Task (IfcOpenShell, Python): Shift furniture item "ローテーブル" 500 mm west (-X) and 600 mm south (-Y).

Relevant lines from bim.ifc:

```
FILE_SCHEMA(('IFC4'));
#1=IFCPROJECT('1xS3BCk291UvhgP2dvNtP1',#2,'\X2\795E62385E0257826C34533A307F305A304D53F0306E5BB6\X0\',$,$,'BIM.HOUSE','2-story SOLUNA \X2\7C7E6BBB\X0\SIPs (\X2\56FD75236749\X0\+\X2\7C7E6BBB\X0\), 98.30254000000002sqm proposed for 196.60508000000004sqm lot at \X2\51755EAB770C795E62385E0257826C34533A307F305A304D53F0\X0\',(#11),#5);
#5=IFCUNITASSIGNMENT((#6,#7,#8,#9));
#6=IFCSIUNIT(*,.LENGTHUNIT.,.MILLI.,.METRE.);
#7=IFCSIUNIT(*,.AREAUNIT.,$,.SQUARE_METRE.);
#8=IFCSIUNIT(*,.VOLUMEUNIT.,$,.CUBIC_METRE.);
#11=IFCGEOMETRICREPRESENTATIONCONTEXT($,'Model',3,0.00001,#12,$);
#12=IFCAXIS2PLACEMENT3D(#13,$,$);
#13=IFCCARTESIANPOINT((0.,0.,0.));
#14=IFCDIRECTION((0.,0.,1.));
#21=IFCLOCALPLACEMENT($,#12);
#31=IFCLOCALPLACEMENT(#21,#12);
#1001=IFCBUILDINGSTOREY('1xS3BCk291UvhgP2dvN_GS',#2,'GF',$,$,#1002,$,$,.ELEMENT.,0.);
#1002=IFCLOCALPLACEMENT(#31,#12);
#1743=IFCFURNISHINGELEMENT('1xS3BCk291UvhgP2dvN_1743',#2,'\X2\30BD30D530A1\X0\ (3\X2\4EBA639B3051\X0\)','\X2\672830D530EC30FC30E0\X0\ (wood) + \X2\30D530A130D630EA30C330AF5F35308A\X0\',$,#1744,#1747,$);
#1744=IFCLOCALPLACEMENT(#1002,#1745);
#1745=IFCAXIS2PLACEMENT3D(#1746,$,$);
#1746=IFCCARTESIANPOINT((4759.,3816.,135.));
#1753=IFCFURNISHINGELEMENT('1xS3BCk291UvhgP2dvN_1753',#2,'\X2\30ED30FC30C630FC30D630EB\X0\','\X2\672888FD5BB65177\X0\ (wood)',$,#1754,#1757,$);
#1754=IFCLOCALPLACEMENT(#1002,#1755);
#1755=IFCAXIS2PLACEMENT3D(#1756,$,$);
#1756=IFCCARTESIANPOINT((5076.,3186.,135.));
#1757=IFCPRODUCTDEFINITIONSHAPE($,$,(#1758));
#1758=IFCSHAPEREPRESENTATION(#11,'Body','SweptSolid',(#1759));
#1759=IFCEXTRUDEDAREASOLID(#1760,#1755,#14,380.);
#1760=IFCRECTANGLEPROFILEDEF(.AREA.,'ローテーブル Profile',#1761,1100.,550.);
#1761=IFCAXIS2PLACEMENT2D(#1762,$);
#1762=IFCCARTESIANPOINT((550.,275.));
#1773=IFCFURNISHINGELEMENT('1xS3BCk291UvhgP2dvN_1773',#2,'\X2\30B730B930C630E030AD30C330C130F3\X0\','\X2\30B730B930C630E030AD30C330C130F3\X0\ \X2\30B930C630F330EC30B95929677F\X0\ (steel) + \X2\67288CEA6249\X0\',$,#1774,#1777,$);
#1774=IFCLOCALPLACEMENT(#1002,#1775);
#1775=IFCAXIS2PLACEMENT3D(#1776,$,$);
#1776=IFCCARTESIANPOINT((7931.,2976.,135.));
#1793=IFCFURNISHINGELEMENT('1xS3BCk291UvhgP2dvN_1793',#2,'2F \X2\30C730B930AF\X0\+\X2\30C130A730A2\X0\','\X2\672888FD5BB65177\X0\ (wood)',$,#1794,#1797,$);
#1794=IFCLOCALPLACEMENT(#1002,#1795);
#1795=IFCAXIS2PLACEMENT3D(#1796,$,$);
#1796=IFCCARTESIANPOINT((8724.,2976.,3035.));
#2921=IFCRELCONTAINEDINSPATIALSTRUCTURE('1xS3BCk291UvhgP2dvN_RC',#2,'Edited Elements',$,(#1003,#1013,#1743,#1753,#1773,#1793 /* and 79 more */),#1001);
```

```python
import ifcopenshell
import ifcopenshell.api.geometry
import ifcopenshell.util.placement
import ifcopenshell.util.unit

model = ifcopenshell.open("bim.ifc")
unit_scale = ifcopenshell.util.unit.calculate_unit_scale(model)

item = model.by_guid("1xS3BCk291UvhgP2dvN_1753")
matrix = ifcopenshell.util.placement.get_local_placement(item.ObjectPlacement)
matrix[0, 3] -= 0.5 / unit_scale
matrix[1, 3] -= 0.6 / unit_scale
ifcopenshell.api.geometry.edit_object_placement(model, product=item, matrix=matrix, is_si=False)

print(ifcopenshell.util.placement.get_local_placement(item.ObjectPlacement).round(3) + 0.0)

model.write("bim_rev.ifc")
```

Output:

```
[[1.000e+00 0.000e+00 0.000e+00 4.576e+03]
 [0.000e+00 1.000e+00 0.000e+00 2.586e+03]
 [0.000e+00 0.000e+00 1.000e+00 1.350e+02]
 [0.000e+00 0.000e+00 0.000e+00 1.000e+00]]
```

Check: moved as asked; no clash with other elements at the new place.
